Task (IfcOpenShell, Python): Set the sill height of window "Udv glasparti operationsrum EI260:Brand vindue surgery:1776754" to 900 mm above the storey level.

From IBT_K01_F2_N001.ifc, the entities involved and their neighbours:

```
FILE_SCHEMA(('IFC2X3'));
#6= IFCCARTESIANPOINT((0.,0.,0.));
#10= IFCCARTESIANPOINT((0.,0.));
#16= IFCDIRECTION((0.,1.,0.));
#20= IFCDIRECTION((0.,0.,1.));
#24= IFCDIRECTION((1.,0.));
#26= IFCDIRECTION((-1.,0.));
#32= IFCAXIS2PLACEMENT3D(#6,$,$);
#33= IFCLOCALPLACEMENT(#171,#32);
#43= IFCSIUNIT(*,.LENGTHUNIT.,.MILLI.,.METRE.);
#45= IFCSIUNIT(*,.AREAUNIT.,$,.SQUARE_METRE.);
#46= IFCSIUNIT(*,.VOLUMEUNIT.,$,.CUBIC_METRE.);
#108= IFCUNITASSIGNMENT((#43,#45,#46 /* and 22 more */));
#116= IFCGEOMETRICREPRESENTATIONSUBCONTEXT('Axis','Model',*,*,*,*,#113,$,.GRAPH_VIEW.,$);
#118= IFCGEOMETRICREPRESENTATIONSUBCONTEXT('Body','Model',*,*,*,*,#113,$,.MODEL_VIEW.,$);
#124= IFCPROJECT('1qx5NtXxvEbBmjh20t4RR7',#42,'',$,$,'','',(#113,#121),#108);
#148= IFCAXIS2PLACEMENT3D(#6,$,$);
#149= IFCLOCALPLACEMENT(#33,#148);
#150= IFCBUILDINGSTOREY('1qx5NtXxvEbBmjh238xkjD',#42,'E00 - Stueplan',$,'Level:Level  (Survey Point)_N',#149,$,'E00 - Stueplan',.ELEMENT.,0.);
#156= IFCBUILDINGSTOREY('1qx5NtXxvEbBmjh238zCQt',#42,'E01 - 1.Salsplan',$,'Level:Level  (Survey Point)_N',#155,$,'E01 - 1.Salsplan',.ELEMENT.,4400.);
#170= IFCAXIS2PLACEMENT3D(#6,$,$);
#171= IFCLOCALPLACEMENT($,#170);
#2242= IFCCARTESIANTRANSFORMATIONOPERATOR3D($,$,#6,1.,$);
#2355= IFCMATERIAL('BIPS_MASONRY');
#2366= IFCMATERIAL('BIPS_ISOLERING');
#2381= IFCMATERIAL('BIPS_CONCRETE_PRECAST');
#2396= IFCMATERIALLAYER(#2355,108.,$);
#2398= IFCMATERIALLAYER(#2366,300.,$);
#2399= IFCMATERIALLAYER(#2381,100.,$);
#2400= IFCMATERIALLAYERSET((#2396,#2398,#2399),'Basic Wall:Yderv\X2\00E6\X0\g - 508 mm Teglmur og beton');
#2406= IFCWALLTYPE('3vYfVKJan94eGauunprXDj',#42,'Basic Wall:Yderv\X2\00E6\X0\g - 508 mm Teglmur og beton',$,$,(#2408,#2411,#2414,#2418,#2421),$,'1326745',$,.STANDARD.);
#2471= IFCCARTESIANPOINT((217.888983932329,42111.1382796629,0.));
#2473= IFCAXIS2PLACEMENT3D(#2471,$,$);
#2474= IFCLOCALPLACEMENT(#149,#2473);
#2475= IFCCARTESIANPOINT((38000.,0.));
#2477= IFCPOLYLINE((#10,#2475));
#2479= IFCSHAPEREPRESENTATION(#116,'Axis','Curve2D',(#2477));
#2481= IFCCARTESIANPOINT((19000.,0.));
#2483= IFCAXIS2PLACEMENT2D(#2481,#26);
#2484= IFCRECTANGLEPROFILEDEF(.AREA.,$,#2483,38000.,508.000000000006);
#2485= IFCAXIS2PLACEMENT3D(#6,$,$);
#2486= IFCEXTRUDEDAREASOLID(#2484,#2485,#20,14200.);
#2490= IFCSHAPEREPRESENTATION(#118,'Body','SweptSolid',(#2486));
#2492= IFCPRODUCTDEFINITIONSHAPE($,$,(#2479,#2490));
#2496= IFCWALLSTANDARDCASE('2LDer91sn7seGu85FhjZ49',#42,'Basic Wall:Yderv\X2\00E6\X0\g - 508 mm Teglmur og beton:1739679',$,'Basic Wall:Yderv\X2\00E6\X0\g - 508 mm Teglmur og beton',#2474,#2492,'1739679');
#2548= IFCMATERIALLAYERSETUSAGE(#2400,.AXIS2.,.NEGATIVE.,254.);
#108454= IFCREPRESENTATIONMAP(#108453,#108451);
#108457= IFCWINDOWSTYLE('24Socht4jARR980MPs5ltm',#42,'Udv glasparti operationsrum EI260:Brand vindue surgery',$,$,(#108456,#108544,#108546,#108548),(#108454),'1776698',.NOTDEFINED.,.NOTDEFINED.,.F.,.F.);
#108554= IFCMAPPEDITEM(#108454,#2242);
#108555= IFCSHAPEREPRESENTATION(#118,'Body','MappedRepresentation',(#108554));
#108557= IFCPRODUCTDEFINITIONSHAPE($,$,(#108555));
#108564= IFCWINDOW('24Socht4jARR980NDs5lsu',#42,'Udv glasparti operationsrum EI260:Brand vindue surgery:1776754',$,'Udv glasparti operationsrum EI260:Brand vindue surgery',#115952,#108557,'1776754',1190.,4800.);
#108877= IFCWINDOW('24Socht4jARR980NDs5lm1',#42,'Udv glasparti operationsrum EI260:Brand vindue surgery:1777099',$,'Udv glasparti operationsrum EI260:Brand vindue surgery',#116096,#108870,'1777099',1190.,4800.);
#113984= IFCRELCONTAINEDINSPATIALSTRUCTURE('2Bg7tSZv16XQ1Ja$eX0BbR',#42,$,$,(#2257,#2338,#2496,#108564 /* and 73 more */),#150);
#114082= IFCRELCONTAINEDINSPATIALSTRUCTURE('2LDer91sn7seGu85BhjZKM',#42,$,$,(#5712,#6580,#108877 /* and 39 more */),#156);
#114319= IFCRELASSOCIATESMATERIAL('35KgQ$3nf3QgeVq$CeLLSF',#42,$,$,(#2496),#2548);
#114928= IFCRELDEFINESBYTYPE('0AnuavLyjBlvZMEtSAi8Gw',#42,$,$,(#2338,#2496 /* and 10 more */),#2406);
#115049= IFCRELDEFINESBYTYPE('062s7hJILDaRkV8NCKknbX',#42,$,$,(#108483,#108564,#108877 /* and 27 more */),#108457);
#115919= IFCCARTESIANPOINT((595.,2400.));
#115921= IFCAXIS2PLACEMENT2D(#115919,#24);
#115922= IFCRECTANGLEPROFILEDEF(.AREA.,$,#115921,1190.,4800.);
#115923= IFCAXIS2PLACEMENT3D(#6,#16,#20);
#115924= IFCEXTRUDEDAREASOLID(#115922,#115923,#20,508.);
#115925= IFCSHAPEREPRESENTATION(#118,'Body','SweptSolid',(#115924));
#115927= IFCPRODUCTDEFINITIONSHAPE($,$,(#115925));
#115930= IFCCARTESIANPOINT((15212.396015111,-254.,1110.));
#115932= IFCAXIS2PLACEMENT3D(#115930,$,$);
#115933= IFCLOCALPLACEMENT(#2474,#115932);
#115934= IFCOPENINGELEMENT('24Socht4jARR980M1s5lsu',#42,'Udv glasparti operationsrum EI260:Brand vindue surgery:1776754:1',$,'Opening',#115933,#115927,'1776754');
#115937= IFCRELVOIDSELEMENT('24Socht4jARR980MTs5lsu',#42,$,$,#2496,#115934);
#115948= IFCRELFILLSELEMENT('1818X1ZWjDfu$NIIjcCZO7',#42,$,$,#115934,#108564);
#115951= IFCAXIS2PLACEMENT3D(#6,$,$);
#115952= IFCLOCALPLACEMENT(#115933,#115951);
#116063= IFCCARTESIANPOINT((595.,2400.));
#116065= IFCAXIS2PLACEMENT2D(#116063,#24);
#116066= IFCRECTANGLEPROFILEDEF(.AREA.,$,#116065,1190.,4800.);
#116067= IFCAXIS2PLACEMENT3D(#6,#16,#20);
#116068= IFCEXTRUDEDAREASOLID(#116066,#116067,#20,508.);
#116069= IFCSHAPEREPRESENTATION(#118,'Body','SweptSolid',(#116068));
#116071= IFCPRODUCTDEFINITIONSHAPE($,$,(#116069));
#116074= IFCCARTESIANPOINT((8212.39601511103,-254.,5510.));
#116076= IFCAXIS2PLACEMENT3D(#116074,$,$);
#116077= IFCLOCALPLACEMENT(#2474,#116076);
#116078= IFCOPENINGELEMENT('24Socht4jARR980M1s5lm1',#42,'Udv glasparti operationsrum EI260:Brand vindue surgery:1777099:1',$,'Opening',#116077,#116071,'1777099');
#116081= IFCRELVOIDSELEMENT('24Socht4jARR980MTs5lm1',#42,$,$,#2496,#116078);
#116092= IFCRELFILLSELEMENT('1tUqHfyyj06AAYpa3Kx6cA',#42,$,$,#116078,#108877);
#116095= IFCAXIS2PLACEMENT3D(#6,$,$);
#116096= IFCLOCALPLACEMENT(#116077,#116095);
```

```python
import numpy as np
import ifcopenshell
import ifcopenshell.api.geometry
import ifcopenshell.geom
import ifcopenshell.util.element
import ifcopenshell.util.placement
import ifcopenshell.util.shape
import ifcopenshell.util.unit

model = ifcopenshell.open("IBT_K01_F2_N001.ifc")
unit_scale = ifcopenshell.util.unit.calculate_unit_scale(model)

window = model.by_guid("24Socht4jARR980NDs5lsu")
opening = window.FillsVoids[0].RelatingOpeningElement
storey = ifcopenshell.util.element.get_container(window, ifc_class="IfcBuildingStorey")
level = ifcopenshell.util.placement.get_local_placement(storey.ObjectPlacement)[2, 3]

# The opening's origin need not be at the sill, so measure its lowest point.
shape = ifcopenshell.geom.create_shape(ifcopenshell.geom.settings(), opening)
bottom = ifcopenshell.util.shape.get_shape_bottom_elevation(shape, shape.geometry) / unit_scale
dz = level + 0.9 / unit_scale - bottom

shift = np.array([0.0, 0.0, dz])
# The window is placed relative to its opening, so it follows when the opening moves.
matrix = ifcopenshell.util.placement.get_local_placement(opening.ObjectPlacement)
matrix[:3, 3] += shift
ifcopenshell.api.geometry.edit_object_placement(
    model, product=opening, matrix=matrix, is_si=False, should_transform_children=True
)

print(f"moved by {dz * unit_scale:+.3f} m")

model.write("IBT_K01_F2_N001_v2.ifc")
```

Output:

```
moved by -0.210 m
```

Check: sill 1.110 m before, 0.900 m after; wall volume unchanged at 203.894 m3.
